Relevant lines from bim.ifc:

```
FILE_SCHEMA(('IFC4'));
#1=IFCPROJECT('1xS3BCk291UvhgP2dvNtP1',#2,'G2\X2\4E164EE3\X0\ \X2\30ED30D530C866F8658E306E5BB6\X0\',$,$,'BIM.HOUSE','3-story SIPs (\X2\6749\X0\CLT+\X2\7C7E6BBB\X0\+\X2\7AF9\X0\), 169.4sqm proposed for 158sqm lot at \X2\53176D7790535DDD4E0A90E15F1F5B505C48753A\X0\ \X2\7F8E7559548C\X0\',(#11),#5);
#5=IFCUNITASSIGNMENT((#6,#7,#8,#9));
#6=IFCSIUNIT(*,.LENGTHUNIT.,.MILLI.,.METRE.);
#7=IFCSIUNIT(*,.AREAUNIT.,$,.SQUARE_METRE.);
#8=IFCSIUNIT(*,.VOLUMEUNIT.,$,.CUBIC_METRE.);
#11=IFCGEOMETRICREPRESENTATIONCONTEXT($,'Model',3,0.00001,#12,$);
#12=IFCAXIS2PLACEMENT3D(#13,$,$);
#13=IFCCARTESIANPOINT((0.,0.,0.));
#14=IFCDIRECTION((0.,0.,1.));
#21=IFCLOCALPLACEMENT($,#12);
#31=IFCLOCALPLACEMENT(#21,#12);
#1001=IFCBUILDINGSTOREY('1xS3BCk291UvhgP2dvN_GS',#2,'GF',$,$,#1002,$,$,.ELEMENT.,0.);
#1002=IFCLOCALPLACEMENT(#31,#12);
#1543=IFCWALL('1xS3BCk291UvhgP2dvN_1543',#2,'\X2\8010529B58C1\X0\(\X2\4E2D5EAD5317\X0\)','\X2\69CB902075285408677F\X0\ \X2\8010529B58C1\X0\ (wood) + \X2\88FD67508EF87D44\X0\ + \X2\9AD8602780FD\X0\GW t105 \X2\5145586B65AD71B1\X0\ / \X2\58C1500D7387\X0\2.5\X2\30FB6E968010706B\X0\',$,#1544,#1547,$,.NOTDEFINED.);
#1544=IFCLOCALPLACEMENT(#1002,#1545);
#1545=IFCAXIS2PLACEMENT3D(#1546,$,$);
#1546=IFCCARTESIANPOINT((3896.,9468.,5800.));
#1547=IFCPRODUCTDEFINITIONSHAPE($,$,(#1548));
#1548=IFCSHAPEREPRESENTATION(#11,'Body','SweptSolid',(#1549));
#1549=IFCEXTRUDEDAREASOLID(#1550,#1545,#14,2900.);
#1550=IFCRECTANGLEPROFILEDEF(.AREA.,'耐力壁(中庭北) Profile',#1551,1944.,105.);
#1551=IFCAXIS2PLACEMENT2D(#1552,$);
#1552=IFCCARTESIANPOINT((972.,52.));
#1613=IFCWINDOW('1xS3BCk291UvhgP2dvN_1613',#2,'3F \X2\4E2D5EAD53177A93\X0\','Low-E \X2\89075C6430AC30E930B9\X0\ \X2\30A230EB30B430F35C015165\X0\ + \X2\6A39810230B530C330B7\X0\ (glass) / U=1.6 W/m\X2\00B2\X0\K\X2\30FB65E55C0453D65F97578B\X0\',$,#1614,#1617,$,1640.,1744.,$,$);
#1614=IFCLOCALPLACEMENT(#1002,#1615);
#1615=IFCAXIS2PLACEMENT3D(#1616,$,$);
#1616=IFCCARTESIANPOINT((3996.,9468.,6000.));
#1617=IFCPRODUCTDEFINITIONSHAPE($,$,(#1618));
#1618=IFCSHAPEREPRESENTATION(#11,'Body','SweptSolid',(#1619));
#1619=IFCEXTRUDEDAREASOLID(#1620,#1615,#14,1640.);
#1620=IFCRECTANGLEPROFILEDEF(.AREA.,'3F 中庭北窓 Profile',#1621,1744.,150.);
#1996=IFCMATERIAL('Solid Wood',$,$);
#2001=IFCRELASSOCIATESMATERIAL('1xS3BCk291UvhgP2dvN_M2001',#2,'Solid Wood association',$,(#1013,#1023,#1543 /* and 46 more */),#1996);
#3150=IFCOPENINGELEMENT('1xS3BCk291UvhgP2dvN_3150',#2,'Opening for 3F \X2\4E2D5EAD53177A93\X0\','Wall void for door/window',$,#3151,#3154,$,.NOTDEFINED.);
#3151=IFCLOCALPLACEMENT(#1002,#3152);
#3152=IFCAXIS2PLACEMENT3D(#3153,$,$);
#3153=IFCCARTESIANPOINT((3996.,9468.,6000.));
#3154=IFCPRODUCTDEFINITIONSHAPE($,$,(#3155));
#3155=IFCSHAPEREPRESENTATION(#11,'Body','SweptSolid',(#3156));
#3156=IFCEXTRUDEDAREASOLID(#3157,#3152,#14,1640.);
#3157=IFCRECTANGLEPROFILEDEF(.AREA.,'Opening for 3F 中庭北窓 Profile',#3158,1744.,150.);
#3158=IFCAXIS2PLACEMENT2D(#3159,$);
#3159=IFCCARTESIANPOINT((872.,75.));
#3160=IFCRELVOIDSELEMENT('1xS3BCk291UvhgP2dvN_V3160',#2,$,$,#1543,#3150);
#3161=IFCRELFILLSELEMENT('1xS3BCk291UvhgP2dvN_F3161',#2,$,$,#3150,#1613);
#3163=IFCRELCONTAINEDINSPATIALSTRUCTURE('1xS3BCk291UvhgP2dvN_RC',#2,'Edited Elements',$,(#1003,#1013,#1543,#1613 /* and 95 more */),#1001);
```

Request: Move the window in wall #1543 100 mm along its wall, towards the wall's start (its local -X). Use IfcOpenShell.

```python
import ifcopenshell
import ifcopenshell.api.geometry
import ifcopenshell.util.placement

model = ifcopenshell.open("bim.ifc")

window = model.by_guid("1xS3BCk291UvhgP2dvN_1613")
opening = window.FillsVoids[0].RelatingOpeningElement
wall = opening.VoidsElements[0].RelatingBuildingElement

wall_matrix = ifcopenshell.util.placement.get_local_placement(wall.ObjectPlacement)
shift = wall_matrix[:3, 0] * -100.0
before = ifcopenshell.util.placement.get_local_placement(window.ObjectPlacement)[:3, 3].copy()

# The window is not placed relative to its opening, so move both.
for product in (opening, window):
    matrix = ifcopenshell.util.placement.get_local_placement(product.ObjectPlacement)
    matrix[:3, 3] += shift
    ifcopenshell.api.geometry.edit_object_placement(model, product=product, matrix=matrix, is_si=False)

after = ifcopenshell.util.placement.get_local_placement(window.ObjectPlacement)[:3, 3]
print("window moved by", (after - before).round(3) + 0.0)

model.write("bim-out.ifc")
```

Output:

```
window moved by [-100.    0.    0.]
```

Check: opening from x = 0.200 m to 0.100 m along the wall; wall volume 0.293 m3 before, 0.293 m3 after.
